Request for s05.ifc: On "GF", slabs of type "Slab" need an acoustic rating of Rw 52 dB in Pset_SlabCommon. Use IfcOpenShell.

First a look at what the model holds.

```python
import ifcopenshell
import ifcopenshell.util.element

model = ifcopenshell.open("s05.ifc")
print(model.schema)
storey = next(s for s in model.by_type("IfcBuildingStorey") if s.Name == "GF")
slabs = [e for e in ifcopenshell.util.element.get_decomposition(storey) if e.is_a("IfcSlab")]
seen = {}
for e in slabs:
    element_type = ifcopenshell.util.element.get_type(e)
    key = (element_type.Name if element_type != e and element_type else None, ifcopenshell.util.element.get_pset(e, "Pset_SlabCommon", "AcousticRating"))
    seen[key] = seen.get(key, 0) + 1
for (name, value), count in sorted(seen.items(), key=str):
    print(count, "x", name, "|", value)
```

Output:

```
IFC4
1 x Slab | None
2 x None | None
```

```python
import ifcopenshell
import ifcopenshell.api.pset
import ifcopenshell.util.element

model = ifcopenshell.open("s05.ifc")

storey = next(s for s in model.by_type("IfcBuildingStorey") if s.Name == "GF")
slabs = [e for e in ifcopenshell.util.element.get_decomposition(storey) if e.is_a("IfcSlab")]

count = 0
for e in slabs:
    element_type = ifcopenshell.util.element.get_type(e)
    if element_type in (None, e) or element_type.Name != "Slab":
        continue
    # add_pset returns the element's existing set when there is one.
    pset = ifcopenshell.api.pset.add_pset(model, product=e, name="Pset_SlabCommon")
    ifcopenshell.api.pset.edit_pset(model, pset=pset, properties={"AcousticRating": "Rw 52 dB"})
    count += 1

print(count, "slabs updated")

model.write("s05_updated.ifc")
```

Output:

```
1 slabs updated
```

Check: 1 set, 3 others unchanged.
